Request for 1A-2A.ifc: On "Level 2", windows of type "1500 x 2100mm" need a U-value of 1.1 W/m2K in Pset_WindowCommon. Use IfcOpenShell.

First a look at what the model holds.

```python
import ifcopenshell
import ifcopenshell.util.element

model = ifcopenshell.open("1A-2A.ifc")
print(model.schema)
storey = next(s for s in model.by_type("IfcBuildingStorey") if s.Name == "Level 2")
windows = [e for e in ifcopenshell.util.element.get_decomposition(storey) if e.is_a("IfcWindow")]
seen = {}
for e in windows:
    element_type = ifcopenshell.util.element.get_type(e)
    key = (element_type.Name if element_type != e and element_type else None, ifcopenshell.util.element.get_pset(e, "Pset_WindowCommon", "ThermalTransmittance"))
    seen[key] = seen.get(key, 0) + 1
for (name, value), count in sorted(seen.items(), key=str):
    print(count, "x", name, "|", value)
```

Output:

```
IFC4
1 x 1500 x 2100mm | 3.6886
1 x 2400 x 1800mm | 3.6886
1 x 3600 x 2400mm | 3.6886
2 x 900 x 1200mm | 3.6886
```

```python
import ifcopenshell
import ifcopenshell.api.pset
import ifcopenshell.util.element

model = ifcopenshell.open("1A-2A.ifc")

storey = next(s for s in model.by_type("IfcBuildingStorey") if s.Name == "Level 2")
windows = [e for e in ifcopenshell.util.element.get_decomposition(storey) if e.is_a("IfcWindow")]

count = 0
for e in windows:
    element_type = ifcopenshell.util.element.get_type(e)
    if element_type in (None, e) or element_type.Name != "1500 x 2100mm":
        continue
    # add_pset returns the element's existing set when there is one.
    pset = ifcopenshell.api.pset.add_pset(model, product=e, name="Pset_WindowCommon")
    ifcopenshell.api.pset.edit_pset(model, pset=pset, properties={"ThermalTransmittance": 1.1})
    count += 1

print(count, "windows updated")

model.write("1A-2A_v2.ifc")
```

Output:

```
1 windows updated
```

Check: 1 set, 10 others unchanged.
